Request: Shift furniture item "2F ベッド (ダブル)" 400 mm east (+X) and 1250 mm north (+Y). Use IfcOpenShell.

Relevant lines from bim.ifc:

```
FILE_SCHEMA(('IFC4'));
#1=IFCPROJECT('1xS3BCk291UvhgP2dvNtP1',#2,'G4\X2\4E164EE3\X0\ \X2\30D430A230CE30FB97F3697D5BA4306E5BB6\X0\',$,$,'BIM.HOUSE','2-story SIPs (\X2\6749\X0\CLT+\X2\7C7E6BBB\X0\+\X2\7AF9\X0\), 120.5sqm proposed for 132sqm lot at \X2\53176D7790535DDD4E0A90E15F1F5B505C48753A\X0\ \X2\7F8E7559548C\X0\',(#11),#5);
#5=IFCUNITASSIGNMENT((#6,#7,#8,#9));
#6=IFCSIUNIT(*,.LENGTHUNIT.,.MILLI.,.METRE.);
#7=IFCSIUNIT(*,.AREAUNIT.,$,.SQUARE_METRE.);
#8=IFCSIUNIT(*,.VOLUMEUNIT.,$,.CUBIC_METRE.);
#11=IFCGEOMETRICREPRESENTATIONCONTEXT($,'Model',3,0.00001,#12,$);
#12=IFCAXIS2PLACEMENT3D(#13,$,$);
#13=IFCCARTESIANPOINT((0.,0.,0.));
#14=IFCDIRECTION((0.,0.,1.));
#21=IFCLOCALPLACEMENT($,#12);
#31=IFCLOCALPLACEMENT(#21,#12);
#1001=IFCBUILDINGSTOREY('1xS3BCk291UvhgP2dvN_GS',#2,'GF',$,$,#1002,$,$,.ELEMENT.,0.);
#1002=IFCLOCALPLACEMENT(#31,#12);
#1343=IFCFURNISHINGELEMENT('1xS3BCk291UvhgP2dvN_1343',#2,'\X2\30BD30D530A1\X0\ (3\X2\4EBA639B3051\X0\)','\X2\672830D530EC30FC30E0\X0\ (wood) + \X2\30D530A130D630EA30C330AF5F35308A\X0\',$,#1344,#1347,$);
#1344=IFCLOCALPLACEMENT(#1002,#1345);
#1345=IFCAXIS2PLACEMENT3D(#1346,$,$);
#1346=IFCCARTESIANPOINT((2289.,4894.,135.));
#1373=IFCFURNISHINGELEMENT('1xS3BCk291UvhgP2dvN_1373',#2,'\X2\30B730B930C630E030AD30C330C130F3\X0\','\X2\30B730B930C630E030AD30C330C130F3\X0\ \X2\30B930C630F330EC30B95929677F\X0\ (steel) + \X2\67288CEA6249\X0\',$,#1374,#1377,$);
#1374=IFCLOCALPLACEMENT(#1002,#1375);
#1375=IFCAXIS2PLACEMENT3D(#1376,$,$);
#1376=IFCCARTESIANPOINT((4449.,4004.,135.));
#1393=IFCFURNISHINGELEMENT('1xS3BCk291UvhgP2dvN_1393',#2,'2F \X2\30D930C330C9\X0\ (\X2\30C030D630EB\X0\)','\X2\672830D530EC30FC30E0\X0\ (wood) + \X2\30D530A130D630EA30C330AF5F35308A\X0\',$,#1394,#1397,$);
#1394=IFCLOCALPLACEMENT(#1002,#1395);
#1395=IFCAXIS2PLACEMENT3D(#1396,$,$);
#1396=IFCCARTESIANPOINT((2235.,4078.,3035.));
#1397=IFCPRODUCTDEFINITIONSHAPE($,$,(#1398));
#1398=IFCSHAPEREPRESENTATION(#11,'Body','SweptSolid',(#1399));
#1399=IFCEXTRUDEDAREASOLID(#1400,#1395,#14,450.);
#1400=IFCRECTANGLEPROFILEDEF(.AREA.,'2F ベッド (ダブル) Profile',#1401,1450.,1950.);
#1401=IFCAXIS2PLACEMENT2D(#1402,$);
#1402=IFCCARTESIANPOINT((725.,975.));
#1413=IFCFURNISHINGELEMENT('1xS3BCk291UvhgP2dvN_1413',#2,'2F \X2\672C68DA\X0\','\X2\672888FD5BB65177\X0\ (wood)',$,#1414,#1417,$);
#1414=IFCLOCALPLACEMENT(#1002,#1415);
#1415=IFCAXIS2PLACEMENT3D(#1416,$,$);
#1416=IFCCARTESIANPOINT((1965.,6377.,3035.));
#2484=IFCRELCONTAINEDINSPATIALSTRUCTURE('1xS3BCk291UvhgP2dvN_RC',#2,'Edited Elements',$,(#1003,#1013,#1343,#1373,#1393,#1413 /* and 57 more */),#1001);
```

```python
import ifcopenshell
import ifcopenshell.api.geometry
import ifcopenshell.util.placement
import ifcopenshell.util.unit

model = ifcopenshell.open("bim.ifc")
unit_scale = ifcopenshell.util.unit.calculate_unit_scale(model)

item = model.by_id(1393)
matrix = ifcopenshell.util.placement.get_local_placement(item.ObjectPlacement)
matrix[0, 3] += 0.4 / unit_scale
matrix[1, 3] += 1.25 / unit_scale
ifcopenshell.api.geometry.edit_object_placement(model, product=item, matrix=matrix, is_si=False)

print(ifcopenshell.util.placement.get_local_placement(item.ObjectPlacement).round(3) + 0.0)

model.write("bim_rev.ifc")
```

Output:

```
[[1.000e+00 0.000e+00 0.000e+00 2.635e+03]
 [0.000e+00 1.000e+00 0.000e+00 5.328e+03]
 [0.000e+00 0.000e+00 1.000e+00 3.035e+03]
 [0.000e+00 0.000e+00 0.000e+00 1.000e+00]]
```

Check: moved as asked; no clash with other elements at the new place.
